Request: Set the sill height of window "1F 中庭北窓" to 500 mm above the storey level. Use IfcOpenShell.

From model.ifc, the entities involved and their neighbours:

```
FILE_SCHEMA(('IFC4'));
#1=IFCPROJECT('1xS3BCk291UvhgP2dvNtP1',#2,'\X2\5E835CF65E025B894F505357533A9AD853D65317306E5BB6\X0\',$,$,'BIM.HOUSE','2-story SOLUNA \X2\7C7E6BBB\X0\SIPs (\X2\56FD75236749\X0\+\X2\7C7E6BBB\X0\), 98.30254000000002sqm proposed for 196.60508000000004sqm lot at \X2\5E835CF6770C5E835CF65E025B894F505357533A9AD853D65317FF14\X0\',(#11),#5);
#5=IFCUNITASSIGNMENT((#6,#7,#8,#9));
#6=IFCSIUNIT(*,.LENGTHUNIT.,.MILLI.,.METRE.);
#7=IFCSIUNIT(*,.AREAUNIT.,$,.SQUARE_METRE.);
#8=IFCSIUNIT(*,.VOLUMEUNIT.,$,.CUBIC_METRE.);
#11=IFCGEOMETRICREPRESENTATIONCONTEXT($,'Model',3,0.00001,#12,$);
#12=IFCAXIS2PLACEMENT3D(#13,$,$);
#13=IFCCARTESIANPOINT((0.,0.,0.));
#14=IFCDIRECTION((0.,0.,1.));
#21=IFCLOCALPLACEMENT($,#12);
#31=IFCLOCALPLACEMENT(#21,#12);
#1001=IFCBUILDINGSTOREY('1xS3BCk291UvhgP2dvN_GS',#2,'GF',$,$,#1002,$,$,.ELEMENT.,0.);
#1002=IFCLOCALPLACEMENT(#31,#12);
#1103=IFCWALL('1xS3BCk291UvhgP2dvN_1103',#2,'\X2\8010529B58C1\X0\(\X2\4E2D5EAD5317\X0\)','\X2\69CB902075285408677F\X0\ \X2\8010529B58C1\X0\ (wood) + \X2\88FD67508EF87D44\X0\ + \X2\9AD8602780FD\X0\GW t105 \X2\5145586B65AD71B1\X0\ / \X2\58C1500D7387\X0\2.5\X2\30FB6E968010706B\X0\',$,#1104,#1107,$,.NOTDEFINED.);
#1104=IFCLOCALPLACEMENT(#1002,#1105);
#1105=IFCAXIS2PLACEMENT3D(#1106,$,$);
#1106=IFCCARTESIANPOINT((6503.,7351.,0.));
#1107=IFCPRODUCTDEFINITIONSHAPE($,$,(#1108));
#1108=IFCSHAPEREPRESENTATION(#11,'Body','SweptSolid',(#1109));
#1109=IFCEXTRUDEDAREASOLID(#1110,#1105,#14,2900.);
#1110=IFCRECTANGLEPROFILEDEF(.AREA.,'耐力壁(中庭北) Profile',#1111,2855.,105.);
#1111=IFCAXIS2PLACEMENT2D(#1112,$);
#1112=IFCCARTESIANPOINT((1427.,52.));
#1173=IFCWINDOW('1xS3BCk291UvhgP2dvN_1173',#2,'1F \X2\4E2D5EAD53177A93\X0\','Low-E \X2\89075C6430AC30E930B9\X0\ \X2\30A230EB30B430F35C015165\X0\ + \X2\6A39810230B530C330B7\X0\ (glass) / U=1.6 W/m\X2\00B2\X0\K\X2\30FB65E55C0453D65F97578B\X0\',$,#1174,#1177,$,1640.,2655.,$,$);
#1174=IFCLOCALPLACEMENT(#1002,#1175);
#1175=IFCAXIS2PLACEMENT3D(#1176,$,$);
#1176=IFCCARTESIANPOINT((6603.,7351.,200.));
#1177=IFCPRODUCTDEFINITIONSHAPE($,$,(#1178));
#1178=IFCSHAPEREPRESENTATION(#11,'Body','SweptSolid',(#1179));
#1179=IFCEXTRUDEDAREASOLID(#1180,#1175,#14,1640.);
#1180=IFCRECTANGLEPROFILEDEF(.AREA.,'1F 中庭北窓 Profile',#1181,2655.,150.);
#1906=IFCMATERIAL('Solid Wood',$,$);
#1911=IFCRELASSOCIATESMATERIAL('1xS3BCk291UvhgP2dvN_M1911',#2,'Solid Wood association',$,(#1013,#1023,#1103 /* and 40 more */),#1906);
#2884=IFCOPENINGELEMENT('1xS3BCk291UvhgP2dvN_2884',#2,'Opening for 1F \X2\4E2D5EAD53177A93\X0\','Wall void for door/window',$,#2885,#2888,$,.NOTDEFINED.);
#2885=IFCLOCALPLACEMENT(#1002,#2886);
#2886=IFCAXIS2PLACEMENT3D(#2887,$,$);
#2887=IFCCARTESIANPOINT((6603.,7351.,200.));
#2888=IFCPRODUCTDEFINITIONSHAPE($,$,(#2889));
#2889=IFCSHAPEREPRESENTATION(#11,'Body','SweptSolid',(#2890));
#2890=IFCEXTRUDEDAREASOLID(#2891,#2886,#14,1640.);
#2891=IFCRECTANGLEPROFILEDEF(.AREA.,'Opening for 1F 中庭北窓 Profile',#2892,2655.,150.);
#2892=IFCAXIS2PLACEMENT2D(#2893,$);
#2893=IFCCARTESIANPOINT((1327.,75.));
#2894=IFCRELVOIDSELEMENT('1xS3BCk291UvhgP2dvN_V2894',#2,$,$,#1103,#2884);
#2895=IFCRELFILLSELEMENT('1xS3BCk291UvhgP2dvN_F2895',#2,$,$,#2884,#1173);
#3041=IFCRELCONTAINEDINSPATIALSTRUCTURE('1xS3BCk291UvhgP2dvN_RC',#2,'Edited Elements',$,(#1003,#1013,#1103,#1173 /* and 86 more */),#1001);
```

```python
import numpy as np
import ifcopenshell
import ifcopenshell.api.geometry
import ifcopenshell.geom
import ifcopenshell.util.element
import ifcopenshell.util.placement
import ifcopenshell.util.shape
import ifcopenshell.util.unit

model = ifcopenshell.open("model.ifc")
unit_scale = ifcopenshell.util.unit.calculate_unit_scale(model)

window = model.by_guid("1xS3BCk291UvhgP2dvN_1173")
opening = window.FillsVoids[0].RelatingOpeningElement
storey = ifcopenshell.util.element.get_container(window, ifc_class="IfcBuildingStorey")
level = ifcopenshell.util.placement.get_local_placement(storey.ObjectPlacement)[2, 3]

# The opening's origin need not be at the sill, so measure its lowest point.
shape = ifcopenshell.geom.create_shape(ifcopenshell.geom.settings(), opening)
bottom = ifcopenshell.util.shape.get_shape_bottom_elevation(shape, shape.geometry) / unit_scale
dz = level + 0.5 / unit_scale - bottom

shift = np.array([0.0, 0.0, dz])
# The window is not placed relative to its opening, so move both.
for product in (opening, window):
    matrix = ifcopenshell.util.placement.get_local_placement(product.ObjectPlacement)
    matrix[:3, 3] += shift
    ifcopenshell.api.geometry.edit_object_placement(model, product=product, matrix=matrix, is_si=False)

print(f"moved by {dz * unit_scale:+.3f} m")

model.write("model-out.ifc")
```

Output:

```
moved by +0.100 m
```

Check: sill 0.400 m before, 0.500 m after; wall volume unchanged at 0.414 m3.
